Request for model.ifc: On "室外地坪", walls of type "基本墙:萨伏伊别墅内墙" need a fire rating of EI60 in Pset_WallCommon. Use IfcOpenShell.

First a look at what the model holds.

```python
import ifcopenshell
import ifcopenshell.util.element

model = ifcopenshell.open("model.ifc")
print(model.schema)
storey = next(s for s in model.by_type("IfcBuildingStorey") if s.Name == "室外地坪")
walls = [e for e in ifcopenshell.util.element.get_decomposition(storey) if e.is_a("IfcWall")]
seen = {}
for e in walls:
    element_type = ifcopenshell.util.element.get_type(e)
    key = (element_type.Name if element_type != e and element_type else None, ifcopenshell.util.element.get_pset(e, "Pset_WallCommon", "FireRating"))
    seen[key] = seen.get(key, 0) + 1
for (name, value), count in sorted(seen.items(), key=str):
    print(count, "x", name, "|", value)
```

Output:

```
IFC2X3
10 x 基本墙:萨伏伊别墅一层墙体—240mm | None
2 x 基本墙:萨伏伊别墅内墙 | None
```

```python
import ifcopenshell
import ifcopenshell.api.pset
import ifcopenshell.util.element

model = ifcopenshell.open("model.ifc")

storey = next(s for s in model.by_type("IfcBuildingStorey") if s.Name == "室外地坪")
walls = [e for e in ifcopenshell.util.element.get_decomposition(storey) if e.is_a("IfcWall")]

count = 0
for e in walls:
    element_type = ifcopenshell.util.element.get_type(e)
    if element_type in (None, e) or element_type.Name != "基本墙:萨伏伊别墅内墙":
        continue
    # add_pset returns the element's existing set when there is one.
    pset = ifcopenshell.api.pset.add_pset(model, product=e, name="Pset_WallCommon")
    ifcopenshell.api.pset.edit_pset(model, pset=pset, properties={"FireRating": "EI60"})
    count += 1

print(count, "walls updated")

model.write("model_v2.ifc")
```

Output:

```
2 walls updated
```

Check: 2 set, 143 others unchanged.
